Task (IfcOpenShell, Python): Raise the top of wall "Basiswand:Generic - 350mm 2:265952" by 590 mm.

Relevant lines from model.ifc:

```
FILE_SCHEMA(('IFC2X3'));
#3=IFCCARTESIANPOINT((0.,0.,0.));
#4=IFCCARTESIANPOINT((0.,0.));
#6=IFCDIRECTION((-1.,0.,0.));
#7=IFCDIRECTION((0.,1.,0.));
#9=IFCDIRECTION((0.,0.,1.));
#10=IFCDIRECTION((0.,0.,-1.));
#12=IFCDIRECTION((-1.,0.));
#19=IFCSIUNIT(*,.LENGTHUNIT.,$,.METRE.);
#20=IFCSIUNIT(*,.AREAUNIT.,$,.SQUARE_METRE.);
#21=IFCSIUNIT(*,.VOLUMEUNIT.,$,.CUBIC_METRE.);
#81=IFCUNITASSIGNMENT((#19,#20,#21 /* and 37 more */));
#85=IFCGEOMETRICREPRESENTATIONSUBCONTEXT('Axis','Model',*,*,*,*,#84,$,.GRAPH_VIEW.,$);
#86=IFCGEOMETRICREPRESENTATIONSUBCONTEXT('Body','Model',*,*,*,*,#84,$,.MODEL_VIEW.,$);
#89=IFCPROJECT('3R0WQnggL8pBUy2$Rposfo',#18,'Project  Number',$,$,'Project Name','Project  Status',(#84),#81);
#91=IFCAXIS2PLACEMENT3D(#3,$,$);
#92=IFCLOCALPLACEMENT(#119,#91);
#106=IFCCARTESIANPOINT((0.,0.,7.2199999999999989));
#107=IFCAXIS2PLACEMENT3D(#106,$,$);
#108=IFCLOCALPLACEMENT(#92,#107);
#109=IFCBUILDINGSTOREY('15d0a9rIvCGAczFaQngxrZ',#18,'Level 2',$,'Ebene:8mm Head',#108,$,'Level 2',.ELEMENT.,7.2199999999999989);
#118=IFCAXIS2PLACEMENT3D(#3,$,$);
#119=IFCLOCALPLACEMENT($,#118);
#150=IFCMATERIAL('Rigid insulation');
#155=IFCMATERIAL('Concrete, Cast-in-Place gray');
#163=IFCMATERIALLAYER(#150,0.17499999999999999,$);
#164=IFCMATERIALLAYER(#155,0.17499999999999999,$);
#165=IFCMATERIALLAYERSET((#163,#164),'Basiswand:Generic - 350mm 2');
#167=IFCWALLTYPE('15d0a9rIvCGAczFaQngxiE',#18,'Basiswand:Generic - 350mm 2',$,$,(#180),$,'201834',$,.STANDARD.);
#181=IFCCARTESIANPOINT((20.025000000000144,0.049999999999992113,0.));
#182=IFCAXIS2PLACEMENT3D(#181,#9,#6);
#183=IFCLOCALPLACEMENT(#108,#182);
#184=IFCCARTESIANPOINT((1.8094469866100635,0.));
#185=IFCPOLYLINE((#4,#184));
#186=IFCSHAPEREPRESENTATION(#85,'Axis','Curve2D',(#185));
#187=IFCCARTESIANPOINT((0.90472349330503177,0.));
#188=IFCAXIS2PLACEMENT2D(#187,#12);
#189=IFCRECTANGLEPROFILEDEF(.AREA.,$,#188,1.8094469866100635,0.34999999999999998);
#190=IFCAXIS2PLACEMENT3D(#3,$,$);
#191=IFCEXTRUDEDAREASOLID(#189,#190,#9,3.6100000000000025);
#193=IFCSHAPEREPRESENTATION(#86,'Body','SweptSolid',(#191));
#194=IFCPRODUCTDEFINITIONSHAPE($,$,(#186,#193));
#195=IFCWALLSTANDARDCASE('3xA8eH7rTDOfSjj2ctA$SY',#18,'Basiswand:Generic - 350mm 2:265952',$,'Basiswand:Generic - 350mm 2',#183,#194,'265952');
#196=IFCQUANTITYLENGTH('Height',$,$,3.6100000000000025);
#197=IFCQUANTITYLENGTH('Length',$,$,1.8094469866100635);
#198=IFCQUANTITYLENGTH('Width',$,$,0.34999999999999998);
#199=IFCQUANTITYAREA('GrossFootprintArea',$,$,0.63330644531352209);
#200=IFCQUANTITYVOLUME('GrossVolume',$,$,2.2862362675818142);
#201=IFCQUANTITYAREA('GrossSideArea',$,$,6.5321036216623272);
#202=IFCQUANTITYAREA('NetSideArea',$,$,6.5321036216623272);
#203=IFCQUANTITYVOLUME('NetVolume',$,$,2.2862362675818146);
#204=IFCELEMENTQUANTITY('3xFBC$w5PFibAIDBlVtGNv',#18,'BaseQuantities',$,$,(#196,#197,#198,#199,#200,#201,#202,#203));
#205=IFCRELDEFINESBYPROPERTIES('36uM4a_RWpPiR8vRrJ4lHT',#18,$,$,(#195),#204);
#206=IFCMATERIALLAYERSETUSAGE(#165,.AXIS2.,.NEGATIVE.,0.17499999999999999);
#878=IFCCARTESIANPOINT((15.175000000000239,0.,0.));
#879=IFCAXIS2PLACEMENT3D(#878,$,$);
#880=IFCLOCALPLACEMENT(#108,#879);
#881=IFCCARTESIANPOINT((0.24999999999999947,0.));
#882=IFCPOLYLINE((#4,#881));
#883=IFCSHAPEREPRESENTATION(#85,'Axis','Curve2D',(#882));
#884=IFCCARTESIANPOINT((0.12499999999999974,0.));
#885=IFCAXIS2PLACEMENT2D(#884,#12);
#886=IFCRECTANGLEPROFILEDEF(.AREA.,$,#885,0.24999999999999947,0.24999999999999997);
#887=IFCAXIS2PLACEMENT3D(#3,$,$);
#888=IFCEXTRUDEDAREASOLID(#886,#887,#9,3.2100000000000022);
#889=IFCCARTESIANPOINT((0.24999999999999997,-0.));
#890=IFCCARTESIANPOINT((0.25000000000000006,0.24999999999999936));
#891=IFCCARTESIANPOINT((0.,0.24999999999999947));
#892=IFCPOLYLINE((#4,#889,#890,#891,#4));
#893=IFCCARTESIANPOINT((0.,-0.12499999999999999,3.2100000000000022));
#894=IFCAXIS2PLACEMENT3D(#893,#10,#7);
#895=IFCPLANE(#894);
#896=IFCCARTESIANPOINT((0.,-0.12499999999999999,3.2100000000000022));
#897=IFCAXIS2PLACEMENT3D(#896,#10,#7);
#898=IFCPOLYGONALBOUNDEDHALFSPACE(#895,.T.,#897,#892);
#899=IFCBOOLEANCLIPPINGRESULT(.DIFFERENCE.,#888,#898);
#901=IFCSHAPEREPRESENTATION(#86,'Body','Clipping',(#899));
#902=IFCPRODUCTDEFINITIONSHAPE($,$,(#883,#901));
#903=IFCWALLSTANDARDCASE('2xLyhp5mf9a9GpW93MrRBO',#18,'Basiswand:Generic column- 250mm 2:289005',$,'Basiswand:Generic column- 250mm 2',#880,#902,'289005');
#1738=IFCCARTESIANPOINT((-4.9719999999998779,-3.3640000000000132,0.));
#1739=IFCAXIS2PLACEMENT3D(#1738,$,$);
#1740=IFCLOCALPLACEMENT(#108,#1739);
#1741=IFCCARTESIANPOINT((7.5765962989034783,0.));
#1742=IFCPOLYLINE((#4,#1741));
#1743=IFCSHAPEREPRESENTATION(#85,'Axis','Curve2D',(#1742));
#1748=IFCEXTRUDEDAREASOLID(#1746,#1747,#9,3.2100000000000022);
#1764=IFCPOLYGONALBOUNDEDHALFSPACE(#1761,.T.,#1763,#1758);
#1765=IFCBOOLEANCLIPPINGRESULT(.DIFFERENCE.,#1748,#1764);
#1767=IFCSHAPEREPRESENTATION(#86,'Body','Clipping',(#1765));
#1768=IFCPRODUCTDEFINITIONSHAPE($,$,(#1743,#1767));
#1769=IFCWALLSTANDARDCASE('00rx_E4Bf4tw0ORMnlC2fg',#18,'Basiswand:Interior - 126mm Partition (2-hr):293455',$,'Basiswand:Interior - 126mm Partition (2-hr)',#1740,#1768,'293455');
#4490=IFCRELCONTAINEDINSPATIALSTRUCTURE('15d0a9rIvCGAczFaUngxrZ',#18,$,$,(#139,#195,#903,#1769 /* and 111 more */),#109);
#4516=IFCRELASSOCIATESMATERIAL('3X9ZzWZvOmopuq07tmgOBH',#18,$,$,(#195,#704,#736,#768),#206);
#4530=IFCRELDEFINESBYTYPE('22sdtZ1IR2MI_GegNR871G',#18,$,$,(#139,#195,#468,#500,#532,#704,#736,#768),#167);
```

```python
import ifcopenshell
import ifcopenshell.api.pset
import ifcopenshell.geom
import ifcopenshell.util.element
import ifcopenshell.util.representation
import ifcopenshell.util.shape
import ifcopenshell.util.unit

model = ifcopenshell.open("model.ifc")
unit_scale = ifcopenshell.util.unit.calculate_unit_scale(model)
area_scale = ifcopenshell.util.unit.calculate_unit_scale(model, "AREAUNIT")
volume_scale = ifcopenshell.util.unit.calculate_unit_scale(model, "VOLUMEUNIT")
settings = ifcopenshell.geom.settings()


def volume(element):
    """Net volume in cubic metres, openings subtracted."""
    shape = ifcopenshell.geom.create_shape(settings, element)
    return ifcopenshell.util.shape.get_volume(shape.geometry)


wall = model.by_guid("3xA8eH7rTDOfSjj2ctA$SY")
before = volume(wall)

body = ifcopenshell.util.representation.get_representation(wall, "Model", "Body")
solid = body.Items[0]
old_height = solid.Depth
solid.Depth += 0.59 / unit_scale
after = volume(wall)
thickness = 0.35  # wall thickness in metres

# Update the stored height, areas and volumes.
qto = model.by_id(ifcopenshell.util.element.get_pset(wall, "BaseQuantities", should_inherit=False)["id"])
ifcopenshell.api.pset.edit_qto(model, qto=qto, properties={
    "Height": solid.Depth,
    "GrossVolume": ifcopenshell.util.element.get_pset(wall, "BaseQuantities", "GrossVolume") * solid.Depth / old_height,
    "GrossSideArea": ifcopenshell.util.element.get_pset(wall, "BaseQuantities", "GrossSideArea") * solid.Depth / old_height,
    "NetSideArea": after / thickness / area_scale,
    "NetVolume": after / volume_scale,
})

print(f"height {old_height:g} -> {solid.Depth:g}, volume {before:.3f} -> {after:.3f} m3")

model.write("model_rev.ifc")
```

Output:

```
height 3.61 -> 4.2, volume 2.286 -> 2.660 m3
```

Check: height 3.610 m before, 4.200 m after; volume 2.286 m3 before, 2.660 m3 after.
